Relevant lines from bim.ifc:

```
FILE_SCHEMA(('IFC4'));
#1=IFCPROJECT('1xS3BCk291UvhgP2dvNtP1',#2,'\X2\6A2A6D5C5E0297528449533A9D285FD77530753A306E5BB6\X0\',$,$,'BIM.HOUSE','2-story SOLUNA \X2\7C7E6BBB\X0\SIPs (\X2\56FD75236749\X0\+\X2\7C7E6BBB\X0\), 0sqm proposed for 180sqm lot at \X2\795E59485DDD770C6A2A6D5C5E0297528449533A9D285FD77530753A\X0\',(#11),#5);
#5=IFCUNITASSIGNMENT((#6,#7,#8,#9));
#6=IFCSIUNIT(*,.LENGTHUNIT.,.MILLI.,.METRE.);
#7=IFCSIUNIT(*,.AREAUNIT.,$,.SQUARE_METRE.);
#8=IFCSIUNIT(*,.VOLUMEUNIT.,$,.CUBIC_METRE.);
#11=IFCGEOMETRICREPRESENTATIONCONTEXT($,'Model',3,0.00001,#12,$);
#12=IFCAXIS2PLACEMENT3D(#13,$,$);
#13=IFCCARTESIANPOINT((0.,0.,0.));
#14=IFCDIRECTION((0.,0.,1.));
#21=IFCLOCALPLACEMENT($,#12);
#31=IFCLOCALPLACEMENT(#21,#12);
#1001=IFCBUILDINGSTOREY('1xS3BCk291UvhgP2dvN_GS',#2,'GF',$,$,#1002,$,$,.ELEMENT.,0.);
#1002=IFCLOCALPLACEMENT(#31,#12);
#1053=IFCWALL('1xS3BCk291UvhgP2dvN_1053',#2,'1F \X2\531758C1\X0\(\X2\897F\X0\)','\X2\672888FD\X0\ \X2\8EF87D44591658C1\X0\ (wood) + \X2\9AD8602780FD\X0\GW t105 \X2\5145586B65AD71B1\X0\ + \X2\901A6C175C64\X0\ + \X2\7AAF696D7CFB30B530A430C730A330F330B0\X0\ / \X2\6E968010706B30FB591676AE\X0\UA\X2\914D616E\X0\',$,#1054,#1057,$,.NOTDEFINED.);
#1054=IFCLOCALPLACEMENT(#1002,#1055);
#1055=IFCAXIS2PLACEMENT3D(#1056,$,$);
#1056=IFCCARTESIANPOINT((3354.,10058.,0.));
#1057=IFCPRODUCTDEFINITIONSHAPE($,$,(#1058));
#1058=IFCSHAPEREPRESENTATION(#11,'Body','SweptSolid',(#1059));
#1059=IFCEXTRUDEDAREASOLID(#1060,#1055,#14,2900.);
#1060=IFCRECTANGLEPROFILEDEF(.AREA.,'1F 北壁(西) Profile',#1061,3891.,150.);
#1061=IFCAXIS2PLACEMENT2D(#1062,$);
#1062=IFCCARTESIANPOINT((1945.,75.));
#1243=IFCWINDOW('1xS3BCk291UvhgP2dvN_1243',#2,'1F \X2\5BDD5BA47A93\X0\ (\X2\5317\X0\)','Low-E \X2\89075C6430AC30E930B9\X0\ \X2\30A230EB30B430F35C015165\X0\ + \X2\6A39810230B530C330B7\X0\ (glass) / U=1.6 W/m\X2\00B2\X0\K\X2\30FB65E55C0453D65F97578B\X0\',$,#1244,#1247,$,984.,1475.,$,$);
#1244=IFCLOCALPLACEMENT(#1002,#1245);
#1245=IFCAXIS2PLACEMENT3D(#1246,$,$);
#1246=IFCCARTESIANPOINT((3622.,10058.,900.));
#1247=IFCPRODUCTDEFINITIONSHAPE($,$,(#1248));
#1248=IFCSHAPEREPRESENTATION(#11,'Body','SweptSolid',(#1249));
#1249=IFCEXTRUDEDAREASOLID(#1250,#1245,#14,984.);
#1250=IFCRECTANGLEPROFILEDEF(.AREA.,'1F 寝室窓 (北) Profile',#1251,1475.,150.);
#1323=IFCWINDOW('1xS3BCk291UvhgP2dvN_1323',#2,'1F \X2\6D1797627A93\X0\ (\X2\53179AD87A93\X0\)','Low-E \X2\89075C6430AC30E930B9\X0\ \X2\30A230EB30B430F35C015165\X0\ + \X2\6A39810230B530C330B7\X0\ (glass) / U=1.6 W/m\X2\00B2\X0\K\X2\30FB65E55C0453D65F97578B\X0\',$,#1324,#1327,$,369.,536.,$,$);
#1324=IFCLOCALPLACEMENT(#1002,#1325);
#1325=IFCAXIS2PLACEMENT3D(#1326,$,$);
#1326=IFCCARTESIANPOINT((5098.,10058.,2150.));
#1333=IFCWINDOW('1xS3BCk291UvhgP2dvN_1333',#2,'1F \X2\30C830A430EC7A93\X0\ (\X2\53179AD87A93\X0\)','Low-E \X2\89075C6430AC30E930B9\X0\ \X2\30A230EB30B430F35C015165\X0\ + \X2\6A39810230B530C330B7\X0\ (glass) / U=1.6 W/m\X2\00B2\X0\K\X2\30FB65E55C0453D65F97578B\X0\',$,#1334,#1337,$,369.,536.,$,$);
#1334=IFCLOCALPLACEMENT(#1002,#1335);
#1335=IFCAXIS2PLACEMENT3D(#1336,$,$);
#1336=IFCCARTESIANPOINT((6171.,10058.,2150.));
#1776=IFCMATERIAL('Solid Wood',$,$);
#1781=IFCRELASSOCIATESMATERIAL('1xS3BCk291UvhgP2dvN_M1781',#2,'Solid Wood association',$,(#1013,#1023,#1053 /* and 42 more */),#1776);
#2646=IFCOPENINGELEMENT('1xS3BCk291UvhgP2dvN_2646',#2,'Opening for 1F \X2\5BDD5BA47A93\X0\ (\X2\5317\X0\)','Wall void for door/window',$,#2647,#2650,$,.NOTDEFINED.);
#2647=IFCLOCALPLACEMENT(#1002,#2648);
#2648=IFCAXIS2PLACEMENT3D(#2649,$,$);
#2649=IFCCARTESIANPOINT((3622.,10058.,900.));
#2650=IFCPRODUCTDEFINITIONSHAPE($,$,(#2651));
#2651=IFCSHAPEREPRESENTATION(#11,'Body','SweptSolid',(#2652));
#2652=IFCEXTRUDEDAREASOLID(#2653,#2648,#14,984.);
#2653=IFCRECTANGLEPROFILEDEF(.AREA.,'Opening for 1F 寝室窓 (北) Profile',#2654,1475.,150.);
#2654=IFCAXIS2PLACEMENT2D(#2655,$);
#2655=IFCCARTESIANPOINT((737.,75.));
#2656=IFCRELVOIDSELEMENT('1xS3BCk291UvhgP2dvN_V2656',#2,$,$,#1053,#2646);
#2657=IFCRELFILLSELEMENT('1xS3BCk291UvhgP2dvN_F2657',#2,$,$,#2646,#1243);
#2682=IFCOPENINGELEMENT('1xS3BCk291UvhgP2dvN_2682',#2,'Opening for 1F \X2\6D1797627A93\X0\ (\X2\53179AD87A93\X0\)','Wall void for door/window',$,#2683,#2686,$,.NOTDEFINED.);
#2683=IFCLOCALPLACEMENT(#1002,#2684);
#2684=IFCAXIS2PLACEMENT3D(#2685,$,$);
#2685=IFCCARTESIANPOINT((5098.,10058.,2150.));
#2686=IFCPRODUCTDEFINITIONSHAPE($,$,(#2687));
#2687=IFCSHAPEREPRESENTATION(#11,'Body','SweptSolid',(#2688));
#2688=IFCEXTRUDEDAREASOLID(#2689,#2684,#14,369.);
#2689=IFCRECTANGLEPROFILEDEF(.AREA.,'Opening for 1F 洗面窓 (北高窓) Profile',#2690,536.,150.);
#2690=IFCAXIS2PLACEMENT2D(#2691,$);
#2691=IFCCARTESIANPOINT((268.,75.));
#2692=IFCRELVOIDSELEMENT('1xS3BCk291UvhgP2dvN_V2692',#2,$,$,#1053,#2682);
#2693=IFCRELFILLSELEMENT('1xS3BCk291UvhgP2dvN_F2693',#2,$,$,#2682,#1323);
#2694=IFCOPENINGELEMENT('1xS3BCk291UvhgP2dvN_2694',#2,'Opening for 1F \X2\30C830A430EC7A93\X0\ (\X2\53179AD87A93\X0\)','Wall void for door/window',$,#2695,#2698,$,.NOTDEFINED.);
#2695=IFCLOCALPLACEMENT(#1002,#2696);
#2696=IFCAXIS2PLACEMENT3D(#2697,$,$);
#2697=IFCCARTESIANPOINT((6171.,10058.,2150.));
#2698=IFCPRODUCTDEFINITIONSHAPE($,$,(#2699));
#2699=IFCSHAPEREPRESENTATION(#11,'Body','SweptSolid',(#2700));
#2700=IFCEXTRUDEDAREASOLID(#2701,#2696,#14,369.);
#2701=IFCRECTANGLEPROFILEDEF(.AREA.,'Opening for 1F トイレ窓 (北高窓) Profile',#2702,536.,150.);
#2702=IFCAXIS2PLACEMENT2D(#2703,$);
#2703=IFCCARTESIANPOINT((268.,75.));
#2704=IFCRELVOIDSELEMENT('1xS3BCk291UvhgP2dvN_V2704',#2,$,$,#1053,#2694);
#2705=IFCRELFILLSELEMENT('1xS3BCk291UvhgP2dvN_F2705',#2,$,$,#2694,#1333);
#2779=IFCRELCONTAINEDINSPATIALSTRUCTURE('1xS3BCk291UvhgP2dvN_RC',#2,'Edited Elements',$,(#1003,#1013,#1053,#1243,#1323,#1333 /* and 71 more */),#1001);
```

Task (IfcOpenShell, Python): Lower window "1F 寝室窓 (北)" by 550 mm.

```python
import numpy as np
import ifcopenshell
import ifcopenshell.api.geometry
import ifcopenshell.util.placement
import ifcopenshell.util.unit

model = ifcopenshell.open("bim.ifc")
unit_scale = ifcopenshell.util.unit.calculate_unit_scale(model)

window = model.by_id(1243)
opening = window.FillsVoids[0].RelatingOpeningElement
dz = -550.0

shift = np.array([0.0, 0.0, dz])
# The window is not placed relative to its opening, so move both.
for product in (opening, window):
    matrix = ifcopenshell.util.placement.get_local_placement(product.ObjectPlacement)
    matrix[:3, 3] += shift
    ifcopenshell.api.geometry.edit_object_placement(model, product=product, matrix=matrix, is_si=False)

print(f"moved by {dz * unit_scale:+.3f} m")

model.write("bim_rev.ifc")
```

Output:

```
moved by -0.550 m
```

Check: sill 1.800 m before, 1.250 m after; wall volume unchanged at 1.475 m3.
